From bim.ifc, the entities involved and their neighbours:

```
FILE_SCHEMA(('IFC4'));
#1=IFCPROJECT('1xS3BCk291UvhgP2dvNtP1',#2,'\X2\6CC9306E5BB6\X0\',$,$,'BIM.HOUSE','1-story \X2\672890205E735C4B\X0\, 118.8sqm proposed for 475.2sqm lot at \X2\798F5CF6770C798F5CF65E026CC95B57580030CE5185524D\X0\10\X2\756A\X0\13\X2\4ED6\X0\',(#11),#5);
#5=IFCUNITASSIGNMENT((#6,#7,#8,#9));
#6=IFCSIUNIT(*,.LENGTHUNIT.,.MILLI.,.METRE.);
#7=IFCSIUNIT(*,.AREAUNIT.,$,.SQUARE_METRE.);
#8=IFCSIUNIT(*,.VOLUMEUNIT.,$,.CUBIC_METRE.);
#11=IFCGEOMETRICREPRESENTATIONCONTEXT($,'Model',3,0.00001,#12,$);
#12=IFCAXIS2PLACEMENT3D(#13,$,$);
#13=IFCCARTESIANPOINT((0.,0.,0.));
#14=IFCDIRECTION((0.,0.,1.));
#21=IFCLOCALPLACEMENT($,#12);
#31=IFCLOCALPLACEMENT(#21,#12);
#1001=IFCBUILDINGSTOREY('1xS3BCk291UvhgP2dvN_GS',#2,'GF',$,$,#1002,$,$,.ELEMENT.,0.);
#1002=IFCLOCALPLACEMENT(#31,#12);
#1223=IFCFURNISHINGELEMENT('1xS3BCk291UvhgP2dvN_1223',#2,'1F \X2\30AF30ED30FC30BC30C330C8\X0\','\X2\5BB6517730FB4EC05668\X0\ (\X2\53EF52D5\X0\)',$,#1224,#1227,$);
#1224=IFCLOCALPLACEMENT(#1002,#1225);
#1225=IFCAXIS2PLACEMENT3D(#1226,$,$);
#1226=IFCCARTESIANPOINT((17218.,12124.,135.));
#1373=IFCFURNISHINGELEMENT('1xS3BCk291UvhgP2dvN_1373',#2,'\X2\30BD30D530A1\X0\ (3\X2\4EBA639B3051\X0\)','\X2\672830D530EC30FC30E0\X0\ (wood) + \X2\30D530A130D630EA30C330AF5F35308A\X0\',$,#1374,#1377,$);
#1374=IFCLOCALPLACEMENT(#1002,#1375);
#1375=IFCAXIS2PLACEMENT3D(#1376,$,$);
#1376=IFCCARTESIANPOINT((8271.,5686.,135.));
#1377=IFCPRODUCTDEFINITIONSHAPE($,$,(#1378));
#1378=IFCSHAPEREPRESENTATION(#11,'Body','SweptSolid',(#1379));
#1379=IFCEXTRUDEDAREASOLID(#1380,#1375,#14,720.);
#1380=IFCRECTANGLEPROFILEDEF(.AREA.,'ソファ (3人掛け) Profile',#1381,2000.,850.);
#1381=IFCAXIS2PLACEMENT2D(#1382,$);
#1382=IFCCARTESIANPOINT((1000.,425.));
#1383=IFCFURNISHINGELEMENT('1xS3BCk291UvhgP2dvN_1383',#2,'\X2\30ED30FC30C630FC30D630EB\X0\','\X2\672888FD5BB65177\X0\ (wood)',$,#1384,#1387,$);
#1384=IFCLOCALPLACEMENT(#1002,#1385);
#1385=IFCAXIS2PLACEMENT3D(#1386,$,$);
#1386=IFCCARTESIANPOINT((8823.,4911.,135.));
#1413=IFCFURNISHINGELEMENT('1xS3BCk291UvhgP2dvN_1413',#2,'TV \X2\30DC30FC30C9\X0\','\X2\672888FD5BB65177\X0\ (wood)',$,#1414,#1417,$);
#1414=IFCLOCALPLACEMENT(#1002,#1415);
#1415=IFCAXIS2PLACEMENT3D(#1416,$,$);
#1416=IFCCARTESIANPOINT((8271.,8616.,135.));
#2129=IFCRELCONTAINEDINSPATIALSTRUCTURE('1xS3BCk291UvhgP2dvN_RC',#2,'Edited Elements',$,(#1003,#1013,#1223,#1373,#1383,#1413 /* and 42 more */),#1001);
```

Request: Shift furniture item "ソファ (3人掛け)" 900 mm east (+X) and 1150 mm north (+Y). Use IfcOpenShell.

```python
import ifcopenshell
import ifcopenshell.api.geometry
import ifcopenshell.util.placement
import ifcopenshell.util.unit

model = ifcopenshell.open("bim.ifc")
unit_scale = ifcopenshell.util.unit.calculate_unit_scale(model)

item = model.by_guid("1xS3BCk291UvhgP2dvN_1373")
matrix = ifcopenshell.util.placement.get_local_placement(item.ObjectPlacement)
matrix[0, 3] += 0.9 / unit_scale
matrix[1, 3] += 1.15 / unit_scale
ifcopenshell.api.geometry.edit_object_placement(model, product=item, matrix=matrix, is_si=False)

print(ifcopenshell.util.placement.get_local_placement(item.ObjectPlacement).round(3) + 0.0)

model.write("bim_updated.ifc")
```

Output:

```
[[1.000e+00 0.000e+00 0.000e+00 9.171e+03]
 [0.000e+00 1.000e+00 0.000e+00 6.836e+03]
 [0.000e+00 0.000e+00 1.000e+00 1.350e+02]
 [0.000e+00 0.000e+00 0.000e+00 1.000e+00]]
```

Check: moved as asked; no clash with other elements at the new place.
